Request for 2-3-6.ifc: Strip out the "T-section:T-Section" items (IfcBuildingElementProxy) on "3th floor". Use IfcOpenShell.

First a look at what the model holds.

```python
import ifcopenshell
import ifcopenshell.util.element

model = ifcopenshell.open("2-3-6.ifc")
print(model.schema)
storey = next(s for s in model.by_type("IfcBuildingStorey") if s.Name == "3th floor")
proxies = [e for e in ifcopenshell.util.element.get_decomposition(storey) if e.is_a("IfcBuildingElementProxy")]
seen = {}
for e in proxies:
    element_type = ifcopenshell.util.element.get_type(e)
    name = element_type.Name if element_type not in (None, e) else None
    seen[name] = seen.get(name, 0) + 1
for name, count in sorted(seen.items(), key=str):
    print(count, "x", name)
```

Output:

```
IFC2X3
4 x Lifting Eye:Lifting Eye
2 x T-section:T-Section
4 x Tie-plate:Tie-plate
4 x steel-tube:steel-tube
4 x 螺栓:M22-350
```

```python
import ifcopenshell
import ifcopenshell.api.root
import ifcopenshell.util.element

model = ifcopenshell.open("2-3-6.ifc")

storey = next(s for s in model.by_type("IfcBuildingStorey") if s.Name == "3th floor")
proxies = [e for e in ifcopenshell.util.element.get_decomposition(storey) if e.is_a("IfcBuildingElementProxy")]
targets = [e for e in proxies if (t := ifcopenshell.util.element.get_type(e)) not in (None, e) and t.Name == "T-section:T-Section"]

for e in targets:
    ifcopenshell.api.root.remove_product(model, product=e)
print(len(targets), "removed")

model.write("2-3-6_rev.ifc")
```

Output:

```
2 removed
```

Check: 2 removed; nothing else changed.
